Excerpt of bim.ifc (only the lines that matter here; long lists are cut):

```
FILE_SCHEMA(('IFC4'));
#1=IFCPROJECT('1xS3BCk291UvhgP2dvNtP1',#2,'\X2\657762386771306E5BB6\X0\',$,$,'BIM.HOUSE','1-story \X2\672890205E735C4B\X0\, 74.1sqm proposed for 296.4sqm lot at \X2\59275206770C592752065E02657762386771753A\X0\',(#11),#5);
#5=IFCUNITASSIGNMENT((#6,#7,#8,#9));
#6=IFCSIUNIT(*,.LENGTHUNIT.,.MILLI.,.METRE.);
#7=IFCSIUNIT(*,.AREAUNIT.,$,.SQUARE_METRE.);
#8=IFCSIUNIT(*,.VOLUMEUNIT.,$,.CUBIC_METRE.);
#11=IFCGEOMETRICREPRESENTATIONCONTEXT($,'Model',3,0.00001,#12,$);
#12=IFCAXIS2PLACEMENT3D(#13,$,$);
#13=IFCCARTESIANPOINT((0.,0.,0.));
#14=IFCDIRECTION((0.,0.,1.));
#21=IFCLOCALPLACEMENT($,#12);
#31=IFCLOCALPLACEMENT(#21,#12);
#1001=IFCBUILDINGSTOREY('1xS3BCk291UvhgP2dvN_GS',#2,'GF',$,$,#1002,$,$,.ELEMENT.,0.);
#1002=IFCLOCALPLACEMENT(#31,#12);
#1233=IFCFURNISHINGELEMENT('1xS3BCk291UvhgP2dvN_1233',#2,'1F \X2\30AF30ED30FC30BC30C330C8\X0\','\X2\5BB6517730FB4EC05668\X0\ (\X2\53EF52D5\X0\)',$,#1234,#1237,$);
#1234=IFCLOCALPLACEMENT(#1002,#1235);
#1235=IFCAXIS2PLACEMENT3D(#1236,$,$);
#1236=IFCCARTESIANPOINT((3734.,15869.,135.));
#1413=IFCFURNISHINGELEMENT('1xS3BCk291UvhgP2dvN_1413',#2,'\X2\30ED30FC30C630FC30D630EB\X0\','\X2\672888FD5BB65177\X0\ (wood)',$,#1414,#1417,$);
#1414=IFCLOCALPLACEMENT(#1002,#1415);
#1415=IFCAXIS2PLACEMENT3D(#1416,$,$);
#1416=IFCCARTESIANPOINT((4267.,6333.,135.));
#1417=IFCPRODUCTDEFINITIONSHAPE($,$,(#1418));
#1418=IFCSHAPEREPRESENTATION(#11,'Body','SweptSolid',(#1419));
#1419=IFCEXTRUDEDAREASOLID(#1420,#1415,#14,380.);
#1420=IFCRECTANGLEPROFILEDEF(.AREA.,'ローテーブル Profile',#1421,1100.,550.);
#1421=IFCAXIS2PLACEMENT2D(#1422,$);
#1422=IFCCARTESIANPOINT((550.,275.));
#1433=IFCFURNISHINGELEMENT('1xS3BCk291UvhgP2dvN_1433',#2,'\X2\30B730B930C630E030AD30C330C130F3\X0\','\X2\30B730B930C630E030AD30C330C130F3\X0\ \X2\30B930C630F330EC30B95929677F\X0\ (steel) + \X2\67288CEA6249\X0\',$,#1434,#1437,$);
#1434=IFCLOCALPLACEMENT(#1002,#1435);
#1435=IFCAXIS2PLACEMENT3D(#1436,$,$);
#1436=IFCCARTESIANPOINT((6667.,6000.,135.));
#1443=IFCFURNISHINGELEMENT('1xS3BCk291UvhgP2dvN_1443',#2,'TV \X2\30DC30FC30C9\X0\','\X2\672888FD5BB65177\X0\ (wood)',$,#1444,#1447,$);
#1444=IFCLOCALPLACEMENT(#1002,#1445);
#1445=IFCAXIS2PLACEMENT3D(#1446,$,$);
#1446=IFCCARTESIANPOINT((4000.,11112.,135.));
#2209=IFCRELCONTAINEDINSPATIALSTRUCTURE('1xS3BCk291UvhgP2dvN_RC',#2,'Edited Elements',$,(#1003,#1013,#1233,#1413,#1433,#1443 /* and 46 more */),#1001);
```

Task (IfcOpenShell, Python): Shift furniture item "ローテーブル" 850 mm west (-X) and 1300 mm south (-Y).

```python
import ifcopenshell
import ifcopenshell.api.geometry
import ifcopenshell.util.placement
import ifcopenshell.util.unit

model = ifcopenshell.open("bim.ifc")
unit_scale = ifcopenshell.util.unit.calculate_unit_scale(model)

item = model.by_guid("1xS3BCk291UvhgP2dvN_1413")
matrix = ifcopenshell.util.placement.get_local_placement(item.ObjectPlacement)
matrix[0, 3] -= 0.85 / unit_scale
matrix[1, 3] -= 1.3 / unit_scale
ifcopenshell.api.geometry.edit_object_placement(model, product=item, matrix=matrix, is_si=False)

print(ifcopenshell.util.placement.get_local_placement(item.ObjectPlacement).round(3) + 0.0)

model.write("bim-out.ifc")
```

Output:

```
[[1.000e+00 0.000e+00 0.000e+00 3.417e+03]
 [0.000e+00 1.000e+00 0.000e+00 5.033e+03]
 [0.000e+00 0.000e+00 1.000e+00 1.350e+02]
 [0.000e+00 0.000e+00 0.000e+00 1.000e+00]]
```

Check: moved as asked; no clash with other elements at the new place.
